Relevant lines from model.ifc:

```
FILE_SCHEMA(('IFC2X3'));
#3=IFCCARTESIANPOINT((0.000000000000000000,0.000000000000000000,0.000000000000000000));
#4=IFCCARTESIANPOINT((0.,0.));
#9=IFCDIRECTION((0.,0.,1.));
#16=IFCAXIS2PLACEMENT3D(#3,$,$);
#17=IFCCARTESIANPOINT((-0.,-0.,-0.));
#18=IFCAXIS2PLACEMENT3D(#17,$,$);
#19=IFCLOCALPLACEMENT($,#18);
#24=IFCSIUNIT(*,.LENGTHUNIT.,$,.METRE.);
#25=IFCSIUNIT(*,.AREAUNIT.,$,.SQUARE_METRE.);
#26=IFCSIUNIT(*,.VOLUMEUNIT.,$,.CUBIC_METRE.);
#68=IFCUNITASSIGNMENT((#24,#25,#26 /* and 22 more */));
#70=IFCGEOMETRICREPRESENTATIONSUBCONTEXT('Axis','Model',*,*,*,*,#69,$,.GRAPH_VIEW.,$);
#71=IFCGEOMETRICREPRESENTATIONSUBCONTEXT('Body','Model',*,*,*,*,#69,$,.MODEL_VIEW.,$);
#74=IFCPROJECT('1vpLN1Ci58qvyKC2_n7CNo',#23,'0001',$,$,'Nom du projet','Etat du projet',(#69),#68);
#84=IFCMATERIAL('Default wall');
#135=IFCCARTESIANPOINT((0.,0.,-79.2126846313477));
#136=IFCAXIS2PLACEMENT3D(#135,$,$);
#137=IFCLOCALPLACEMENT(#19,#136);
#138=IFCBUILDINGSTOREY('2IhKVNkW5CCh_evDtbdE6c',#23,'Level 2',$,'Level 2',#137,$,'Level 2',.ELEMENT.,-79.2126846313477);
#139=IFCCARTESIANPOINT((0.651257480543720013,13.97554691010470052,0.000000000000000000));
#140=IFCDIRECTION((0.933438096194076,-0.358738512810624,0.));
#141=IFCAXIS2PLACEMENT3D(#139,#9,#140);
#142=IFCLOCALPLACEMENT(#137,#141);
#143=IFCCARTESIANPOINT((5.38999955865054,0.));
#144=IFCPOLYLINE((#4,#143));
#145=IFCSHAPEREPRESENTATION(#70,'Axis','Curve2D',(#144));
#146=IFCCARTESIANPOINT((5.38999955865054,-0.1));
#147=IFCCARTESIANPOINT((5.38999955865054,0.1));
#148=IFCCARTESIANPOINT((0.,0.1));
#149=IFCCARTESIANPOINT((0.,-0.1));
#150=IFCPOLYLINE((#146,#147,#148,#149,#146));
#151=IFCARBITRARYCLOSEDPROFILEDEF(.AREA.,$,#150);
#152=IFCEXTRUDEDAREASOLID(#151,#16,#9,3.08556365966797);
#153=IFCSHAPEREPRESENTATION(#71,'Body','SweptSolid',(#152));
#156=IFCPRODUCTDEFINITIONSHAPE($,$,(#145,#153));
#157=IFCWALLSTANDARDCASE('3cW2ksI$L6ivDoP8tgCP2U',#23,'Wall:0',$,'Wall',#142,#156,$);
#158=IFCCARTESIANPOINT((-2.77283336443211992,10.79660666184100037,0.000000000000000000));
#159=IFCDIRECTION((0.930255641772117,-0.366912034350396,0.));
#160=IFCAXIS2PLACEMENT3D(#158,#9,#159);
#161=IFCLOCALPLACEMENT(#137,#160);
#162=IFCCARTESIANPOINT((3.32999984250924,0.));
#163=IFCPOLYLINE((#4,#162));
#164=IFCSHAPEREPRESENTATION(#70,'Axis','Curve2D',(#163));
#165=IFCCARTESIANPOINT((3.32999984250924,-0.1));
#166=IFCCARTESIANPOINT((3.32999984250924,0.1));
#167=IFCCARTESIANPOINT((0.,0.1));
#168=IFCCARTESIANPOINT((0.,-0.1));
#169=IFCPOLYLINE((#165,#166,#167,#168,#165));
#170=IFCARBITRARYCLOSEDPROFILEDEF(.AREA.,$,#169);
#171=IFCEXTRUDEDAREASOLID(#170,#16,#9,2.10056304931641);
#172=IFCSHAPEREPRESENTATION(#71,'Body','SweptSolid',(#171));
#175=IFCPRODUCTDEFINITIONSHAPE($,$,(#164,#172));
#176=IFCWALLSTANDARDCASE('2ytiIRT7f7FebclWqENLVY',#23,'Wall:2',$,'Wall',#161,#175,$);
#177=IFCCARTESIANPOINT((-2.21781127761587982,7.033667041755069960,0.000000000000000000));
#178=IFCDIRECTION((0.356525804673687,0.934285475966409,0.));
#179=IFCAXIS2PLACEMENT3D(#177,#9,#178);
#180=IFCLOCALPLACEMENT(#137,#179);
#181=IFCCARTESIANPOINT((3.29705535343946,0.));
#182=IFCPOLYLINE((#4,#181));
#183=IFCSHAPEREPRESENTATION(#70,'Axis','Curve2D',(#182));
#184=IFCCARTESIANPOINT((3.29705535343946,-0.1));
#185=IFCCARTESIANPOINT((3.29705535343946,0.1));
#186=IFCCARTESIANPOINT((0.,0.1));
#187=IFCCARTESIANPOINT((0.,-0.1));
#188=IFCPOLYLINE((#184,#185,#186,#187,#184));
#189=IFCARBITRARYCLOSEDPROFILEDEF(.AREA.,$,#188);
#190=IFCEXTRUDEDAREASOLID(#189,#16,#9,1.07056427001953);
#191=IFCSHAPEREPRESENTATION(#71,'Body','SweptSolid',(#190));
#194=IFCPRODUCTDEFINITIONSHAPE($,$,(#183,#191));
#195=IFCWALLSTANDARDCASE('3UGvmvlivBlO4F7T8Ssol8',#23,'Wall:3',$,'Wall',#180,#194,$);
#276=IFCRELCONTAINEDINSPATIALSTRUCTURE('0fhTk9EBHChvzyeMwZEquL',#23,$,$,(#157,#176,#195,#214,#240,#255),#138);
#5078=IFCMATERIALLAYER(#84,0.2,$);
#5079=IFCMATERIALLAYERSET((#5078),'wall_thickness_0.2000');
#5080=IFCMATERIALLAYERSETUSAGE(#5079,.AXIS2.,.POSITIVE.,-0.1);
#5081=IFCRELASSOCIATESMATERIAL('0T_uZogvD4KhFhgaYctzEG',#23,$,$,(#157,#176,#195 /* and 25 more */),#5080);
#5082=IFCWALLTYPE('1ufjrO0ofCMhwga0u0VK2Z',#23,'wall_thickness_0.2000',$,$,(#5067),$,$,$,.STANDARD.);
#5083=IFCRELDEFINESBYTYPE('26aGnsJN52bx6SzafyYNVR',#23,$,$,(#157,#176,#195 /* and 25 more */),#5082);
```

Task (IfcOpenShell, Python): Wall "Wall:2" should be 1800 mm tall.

```python
import ifcopenshell
import ifcopenshell.geom
import ifcopenshell.util.representation
import ifcopenshell.util.shape

model = ifcopenshell.open("model.ifc")
settings = ifcopenshell.geom.settings()


def volume(element):
    """Net volume in cubic metres, openings subtracted."""
    shape = ifcopenshell.geom.create_shape(settings, element)
    return ifcopenshell.util.shape.get_volume(shape.geometry)


wall = model.by_guid("2ytiIRT7f7FebclWqENLVY")
before = volume(wall)

body = ifcopenshell.util.representation.get_representation(wall, "Model", "Body")
solid = body.Items[0]
old_height = solid.Depth
solid.Depth = 1.8
after = volume(wall)

print(f"height {old_height:g} -> {solid.Depth:g}, volume {before:.3f} -> {after:.3f} m3")

model.write("model_edited.ifc")
```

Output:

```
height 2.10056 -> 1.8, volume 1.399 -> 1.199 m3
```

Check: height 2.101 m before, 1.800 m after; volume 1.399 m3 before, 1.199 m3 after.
